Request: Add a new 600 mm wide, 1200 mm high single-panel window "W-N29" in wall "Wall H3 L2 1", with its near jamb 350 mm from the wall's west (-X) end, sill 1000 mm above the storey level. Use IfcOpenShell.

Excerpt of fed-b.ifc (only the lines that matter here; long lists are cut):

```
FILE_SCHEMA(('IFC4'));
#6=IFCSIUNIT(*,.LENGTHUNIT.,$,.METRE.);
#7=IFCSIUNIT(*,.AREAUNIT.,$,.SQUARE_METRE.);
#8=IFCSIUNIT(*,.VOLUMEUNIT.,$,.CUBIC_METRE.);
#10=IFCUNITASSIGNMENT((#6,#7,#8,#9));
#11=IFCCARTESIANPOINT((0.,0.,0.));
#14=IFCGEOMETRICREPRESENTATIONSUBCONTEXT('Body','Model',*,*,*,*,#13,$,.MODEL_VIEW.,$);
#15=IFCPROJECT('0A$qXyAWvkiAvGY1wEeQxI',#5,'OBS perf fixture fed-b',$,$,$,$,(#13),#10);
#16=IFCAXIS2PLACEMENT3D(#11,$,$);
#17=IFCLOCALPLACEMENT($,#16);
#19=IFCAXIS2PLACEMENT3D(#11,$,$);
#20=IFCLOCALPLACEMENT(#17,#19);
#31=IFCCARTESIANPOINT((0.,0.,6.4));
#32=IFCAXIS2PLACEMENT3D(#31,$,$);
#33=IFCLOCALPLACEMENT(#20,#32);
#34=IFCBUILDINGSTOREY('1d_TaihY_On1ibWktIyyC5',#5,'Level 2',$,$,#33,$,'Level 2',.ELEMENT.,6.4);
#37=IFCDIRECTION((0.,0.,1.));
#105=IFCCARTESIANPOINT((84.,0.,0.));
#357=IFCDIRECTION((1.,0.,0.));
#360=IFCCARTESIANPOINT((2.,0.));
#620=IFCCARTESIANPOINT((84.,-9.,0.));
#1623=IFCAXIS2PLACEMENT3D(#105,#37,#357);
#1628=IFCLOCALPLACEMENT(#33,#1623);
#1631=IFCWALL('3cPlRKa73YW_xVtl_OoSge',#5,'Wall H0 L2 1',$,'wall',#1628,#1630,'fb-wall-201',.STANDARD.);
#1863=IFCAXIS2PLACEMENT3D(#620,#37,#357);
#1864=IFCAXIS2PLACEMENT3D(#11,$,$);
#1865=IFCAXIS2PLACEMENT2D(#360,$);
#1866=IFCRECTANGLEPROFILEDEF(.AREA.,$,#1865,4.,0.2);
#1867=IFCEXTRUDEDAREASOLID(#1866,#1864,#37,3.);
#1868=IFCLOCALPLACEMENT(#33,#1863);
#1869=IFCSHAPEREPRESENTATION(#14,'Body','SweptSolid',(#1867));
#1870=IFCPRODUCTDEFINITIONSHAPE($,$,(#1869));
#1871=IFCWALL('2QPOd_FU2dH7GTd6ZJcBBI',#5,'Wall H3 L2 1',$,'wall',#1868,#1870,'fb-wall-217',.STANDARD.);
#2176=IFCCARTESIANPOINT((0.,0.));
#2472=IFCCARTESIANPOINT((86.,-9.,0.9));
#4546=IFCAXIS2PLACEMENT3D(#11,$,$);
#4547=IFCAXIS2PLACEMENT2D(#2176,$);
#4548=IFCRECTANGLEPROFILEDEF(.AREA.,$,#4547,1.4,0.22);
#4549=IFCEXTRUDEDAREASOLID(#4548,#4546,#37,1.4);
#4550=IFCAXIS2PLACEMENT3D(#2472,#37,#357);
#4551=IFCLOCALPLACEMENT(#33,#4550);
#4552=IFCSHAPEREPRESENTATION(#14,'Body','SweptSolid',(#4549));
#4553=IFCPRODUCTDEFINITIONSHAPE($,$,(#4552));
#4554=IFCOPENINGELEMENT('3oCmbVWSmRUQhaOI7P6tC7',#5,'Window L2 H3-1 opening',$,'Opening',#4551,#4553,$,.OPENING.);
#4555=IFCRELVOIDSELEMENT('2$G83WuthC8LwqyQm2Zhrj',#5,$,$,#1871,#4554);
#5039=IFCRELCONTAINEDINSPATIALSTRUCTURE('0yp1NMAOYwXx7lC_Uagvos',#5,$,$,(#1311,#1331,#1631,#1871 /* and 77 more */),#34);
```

```python
import numpy as np
import ifcopenshell
import ifcopenshell.api.feature
import ifcopenshell.api.geometry
import ifcopenshell.api.root
import ifcopenshell.api.spatial
import ifcopenshell.geom
import ifcopenshell.util.element
import ifcopenshell.util.placement
import ifcopenshell.util.representation
import ifcopenshell.util.shape
import ifcopenshell.util.unit

model = ifcopenshell.open("fed-b.ifc")
unit_scale = ifcopenshell.util.unit.calculate_unit_scale(model)
settings = ifcopenshell.geom.settings()


def volume(element):
    """Net volume in cubic metres, openings subtracted."""
    shape = ifcopenshell.geom.create_shape(settings, element)
    return ifcopenshell.util.shape.get_volume(shape.geometry)


wall = model.by_guid("2QPOd_FU2dH7GTd6ZJcBBI")
storey = ifcopenshell.util.element.get_container(wall, ifc_class="IfcBuildingStorey")
context = ifcopenshell.util.representation.get_context(model, "Model", "Body", "MODEL_VIEW")
before = volume(wall)

width, height, from_end, sill = 0.6, 1.2, 0.35, 1  # metres

# The wall runs along its own X axis, and the end named is its -X end.
wall_shape = ifcopenshell.geom.create_shape(settings, wall)
x, y, z = ifcopenshell.util.shape.get_vertices(wall_shape.geometry).T
start = x.min() + from_end
face, thickness = float(y.min()), float(y.max() - y.min())
wall_matrix = ifcopenshell.util.placement.get_local_placement(wall.ObjectPlacement)
level = ifcopenshell.util.placement.get_local_placement(storey.ObjectPlacement)[2, 3]


def in_wall(x, y):
    """Placement at x, y metres in the wall's axes, at sill height."""
    matrix = wall_matrix.copy()
    matrix[:, 3] = wall_matrix @ np.array([x / unit_scale, y / unit_scale, 0.0, 1.0])
    matrix[2, 3] = level + sill / unit_scale
    return matrix


# Opening: a box that overshoots both wall faces by 50 mm.
opening = ifcopenshell.api.root.create_entity(model, ifc_class="IfcOpeningElement", predefined_type="OPENING")
box = ifcopenshell.api.geometry.add_wall_representation(
    model, context=context, length=width, height=height, thickness=thickness + 0.1
)
ifcopenshell.api.geometry.assign_representation(model, product=opening, representation=box)
ifcopenshell.api.geometry.edit_object_placement(model, product=opening, matrix=in_wall(start, face - 0.05), is_si=False)
ifcopenshell.api.feature.add_feature(model, feature=opening, element=wall)

window = ifcopenshell.api.root.create_entity(model, ifc_class="IfcWindow", name="W-N29", predefined_type="WINDOW")
window.OverallWidth, window.OverallHeight = width / unit_scale, height / unit_scale
window.PartitioningType = "SINGLE_PANEL"
body = ifcopenshell.api.geometry.add_window_representation(
    model,
    context=context,
    overall_width=window.OverallWidth,
    overall_height=window.OverallHeight,
    partition_type="SINGLE_PANEL",
)
ifcopenshell.api.geometry.assign_representation(model, product=window, representation=body)
ifcopenshell.api.spatial.assign_container(model, products=[window], relating_structure=storey)
ifcopenshell.api.feature.add_filling(model, opening=opening, element=window)

# Centre the window in the wall's thickness.
ifcopenshell.api.geometry.edit_object_placement(model, product=window, matrix=in_wall(start, face), is_si=False)
window_shape = ifcopenshell.geom.create_shape(settings, window)
depth = ifcopenshell.util.shape.get_vertices(window_shape.geometry)[:, 1]
offset = face + thickness / 2 - (depth.min() + depth.max()) / 2
ifcopenshell.api.geometry.edit_object_placement(model, product=window, matrix=in_wall(start, offset), is_si=False)

after = volume(wall)

print(f"wall volume {before:.3f} -> {after:.3f} m3")

model.write("fed-b_edited.ifc")
```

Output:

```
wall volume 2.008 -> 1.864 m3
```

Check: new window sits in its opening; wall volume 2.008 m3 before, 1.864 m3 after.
